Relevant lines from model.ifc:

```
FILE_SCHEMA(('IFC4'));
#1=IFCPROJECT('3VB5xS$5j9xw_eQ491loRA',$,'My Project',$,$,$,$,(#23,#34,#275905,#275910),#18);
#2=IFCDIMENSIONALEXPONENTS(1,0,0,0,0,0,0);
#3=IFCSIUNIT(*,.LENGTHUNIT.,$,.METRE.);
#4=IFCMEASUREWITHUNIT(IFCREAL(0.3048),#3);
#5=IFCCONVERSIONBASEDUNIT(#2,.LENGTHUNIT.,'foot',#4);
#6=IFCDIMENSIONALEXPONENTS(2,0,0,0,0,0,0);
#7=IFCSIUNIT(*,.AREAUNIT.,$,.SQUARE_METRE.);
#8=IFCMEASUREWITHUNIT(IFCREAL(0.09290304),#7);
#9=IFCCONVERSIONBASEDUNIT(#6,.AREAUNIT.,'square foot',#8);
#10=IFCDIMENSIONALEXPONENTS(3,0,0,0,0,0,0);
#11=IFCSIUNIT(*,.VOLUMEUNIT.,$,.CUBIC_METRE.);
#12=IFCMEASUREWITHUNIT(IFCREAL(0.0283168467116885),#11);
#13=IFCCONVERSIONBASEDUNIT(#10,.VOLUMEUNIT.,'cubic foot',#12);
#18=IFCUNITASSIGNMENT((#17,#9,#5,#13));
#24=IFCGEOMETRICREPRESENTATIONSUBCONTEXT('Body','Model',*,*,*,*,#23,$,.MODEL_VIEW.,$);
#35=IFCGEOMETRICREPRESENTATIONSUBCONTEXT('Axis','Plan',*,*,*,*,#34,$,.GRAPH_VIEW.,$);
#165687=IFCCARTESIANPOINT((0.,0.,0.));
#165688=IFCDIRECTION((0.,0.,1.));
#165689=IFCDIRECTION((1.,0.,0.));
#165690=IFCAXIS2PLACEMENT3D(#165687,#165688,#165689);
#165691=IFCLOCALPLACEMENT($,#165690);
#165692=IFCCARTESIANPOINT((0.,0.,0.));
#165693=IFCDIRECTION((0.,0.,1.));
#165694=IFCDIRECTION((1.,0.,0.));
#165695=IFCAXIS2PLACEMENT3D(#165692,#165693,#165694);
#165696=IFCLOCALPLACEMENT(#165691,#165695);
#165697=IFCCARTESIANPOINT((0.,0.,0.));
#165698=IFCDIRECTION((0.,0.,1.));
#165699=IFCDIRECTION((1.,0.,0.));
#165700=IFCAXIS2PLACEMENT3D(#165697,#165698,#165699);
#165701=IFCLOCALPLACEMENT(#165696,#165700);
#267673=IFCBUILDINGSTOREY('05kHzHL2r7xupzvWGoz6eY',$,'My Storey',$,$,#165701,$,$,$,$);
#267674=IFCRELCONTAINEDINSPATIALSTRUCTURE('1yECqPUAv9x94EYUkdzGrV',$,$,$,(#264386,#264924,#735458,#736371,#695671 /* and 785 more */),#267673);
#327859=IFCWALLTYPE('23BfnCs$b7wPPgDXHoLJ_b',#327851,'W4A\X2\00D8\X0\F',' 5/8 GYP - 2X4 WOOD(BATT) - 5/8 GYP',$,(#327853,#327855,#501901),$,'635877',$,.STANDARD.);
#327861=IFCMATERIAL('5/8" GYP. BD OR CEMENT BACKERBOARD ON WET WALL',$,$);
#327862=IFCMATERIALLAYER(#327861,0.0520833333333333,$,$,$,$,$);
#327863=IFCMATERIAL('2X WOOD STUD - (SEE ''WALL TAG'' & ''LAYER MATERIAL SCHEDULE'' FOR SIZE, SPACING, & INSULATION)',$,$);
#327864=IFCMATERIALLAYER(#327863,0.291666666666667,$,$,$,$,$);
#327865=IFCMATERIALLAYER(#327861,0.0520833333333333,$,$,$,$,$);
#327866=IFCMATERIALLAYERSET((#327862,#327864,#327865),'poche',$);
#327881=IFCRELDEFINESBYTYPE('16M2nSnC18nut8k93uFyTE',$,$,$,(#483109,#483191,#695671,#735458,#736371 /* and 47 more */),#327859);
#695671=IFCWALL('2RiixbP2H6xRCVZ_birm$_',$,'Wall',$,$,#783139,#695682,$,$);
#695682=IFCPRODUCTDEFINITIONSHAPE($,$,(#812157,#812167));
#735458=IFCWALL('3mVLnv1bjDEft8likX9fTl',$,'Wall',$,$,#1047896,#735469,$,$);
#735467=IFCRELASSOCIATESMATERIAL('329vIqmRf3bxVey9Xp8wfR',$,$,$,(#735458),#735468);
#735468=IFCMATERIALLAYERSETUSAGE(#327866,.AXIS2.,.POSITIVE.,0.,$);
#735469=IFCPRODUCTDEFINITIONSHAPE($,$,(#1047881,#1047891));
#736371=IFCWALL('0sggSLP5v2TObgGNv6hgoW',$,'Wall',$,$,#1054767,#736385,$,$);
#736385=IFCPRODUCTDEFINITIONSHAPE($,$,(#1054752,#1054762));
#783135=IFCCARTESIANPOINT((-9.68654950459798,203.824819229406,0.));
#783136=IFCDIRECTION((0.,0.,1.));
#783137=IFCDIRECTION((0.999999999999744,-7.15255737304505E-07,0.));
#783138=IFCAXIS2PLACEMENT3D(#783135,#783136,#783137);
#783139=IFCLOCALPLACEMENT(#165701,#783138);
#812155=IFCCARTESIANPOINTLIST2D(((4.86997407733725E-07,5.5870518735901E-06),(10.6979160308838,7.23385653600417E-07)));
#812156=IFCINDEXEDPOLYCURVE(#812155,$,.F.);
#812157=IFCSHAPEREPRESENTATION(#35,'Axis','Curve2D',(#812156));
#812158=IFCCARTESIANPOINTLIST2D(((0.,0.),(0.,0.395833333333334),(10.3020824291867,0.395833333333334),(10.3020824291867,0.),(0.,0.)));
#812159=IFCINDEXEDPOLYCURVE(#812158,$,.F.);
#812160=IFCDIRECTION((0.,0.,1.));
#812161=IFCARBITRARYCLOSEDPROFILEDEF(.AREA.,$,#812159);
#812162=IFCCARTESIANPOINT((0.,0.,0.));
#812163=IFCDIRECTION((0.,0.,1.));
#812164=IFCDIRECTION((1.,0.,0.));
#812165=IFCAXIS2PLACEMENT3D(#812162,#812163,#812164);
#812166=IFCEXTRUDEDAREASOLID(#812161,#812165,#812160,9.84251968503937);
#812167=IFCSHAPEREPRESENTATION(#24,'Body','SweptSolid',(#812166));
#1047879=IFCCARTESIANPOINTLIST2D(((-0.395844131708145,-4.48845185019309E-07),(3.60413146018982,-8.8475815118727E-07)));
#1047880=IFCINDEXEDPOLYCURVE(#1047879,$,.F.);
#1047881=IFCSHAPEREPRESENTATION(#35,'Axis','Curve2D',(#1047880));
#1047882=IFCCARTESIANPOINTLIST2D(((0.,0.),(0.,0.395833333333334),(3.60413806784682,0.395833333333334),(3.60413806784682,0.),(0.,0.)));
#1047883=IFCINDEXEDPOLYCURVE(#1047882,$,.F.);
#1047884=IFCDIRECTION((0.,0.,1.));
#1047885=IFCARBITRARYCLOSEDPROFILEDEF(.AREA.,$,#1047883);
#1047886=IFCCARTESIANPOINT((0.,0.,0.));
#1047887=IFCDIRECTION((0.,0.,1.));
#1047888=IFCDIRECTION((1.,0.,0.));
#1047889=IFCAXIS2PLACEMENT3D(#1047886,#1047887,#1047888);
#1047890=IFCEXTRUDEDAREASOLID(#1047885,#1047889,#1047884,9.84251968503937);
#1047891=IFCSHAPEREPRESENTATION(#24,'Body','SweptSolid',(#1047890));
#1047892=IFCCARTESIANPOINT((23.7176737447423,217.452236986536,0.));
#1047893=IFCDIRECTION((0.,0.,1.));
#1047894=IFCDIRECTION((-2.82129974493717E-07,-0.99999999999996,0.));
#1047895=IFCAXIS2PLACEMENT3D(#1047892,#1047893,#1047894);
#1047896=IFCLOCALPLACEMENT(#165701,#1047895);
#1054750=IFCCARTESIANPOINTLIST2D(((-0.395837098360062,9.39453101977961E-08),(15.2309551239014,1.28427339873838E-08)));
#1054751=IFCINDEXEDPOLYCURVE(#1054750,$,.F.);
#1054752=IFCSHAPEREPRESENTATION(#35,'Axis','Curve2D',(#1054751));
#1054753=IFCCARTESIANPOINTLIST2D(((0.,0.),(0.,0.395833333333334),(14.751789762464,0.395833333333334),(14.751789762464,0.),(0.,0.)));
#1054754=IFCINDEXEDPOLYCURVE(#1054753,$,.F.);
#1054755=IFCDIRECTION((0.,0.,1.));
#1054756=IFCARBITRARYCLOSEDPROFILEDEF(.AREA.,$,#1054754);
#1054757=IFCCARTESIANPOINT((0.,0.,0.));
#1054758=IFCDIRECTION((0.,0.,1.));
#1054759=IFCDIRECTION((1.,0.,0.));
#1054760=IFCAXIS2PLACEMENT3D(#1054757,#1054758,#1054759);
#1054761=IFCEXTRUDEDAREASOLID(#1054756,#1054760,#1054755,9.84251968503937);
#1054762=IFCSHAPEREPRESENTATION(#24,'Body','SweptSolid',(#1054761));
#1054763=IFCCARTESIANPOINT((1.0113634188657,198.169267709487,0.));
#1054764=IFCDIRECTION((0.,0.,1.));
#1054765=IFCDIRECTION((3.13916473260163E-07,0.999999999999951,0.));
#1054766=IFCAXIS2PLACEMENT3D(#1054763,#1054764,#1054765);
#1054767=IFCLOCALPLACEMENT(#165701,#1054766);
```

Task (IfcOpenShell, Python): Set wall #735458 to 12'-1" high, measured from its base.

```python
import ifcopenshell
import ifcopenshell.geom
import ifcopenshell.util.representation
import ifcopenshell.util.shape
import ifcopenshell.util.unit

model = ifcopenshell.open("model.ifc")
unit_scale = ifcopenshell.util.unit.calculate_unit_scale(model)
settings = ifcopenshell.geom.settings()


def volume(element):
    """Net volume in cubic metres, openings subtracted."""
    shape = ifcopenshell.geom.create_shape(settings, element)
    return ifcopenshell.util.shape.get_volume(shape.geometry)


wall = model.by_guid("3mVLnv1bjDEft8likX9fTl")
before = volume(wall)

body = ifcopenshell.util.representation.get_representation(wall, "Model", "Body")
solid = body.Items[0]
old_height = solid.Depth
solid.Depth = 145 * 0.0254 / unit_scale
after = volume(wall)

print(f"height {old_height:g} -> {solid.Depth:g}, volume {before:.3f} -> {after:.3f} m3")

model.write("model_v2.ifc")
```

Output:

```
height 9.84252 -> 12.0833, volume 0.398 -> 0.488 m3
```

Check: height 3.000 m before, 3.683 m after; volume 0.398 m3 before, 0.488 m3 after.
